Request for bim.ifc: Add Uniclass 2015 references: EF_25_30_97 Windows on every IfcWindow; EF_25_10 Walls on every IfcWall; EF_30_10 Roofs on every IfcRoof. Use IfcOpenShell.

First a look at what the model holds.

```python
import ifcopenshell

model = ifcopenshell.open("bim.ifc")
print(model.schema)
print("classifications:", [c.Name for c in model.by_type("IfcClassification")])
for ifc_class in ("IfcDoor", "IfcRoof", "IfcStair", "IfcWall", "IfcWindow"):
    print(ifc_class, len(model.by_type(ifc_class)))
```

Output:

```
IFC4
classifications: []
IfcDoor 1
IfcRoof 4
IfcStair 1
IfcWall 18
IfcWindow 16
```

```python
import ifcopenshell
import ifcopenshell.api.classification

model = ifcopenshell.open("bim.ifc")

system = ifcopenshell.api.classification.add_classification(model, classification="Uniclass 2015")

codes = {
    "IfcWindow": ("EF_25_30_97", "Windows"),
    "IfcWall": ("EF_25_10", "Walls"),
    "IfcRoof": ("EF_30_10", "Roofs"),
}
for ifc_class, (code, name) in codes.items():
    products = model.by_type(ifc_class)
    ifcopenshell.api.classification.add_reference(
        model, products=products, classification=system, identification=code, name=name
    )
    print(code, len(products))

model.write("bim_v2.ifc")
```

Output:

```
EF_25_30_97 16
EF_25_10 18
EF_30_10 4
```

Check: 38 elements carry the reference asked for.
